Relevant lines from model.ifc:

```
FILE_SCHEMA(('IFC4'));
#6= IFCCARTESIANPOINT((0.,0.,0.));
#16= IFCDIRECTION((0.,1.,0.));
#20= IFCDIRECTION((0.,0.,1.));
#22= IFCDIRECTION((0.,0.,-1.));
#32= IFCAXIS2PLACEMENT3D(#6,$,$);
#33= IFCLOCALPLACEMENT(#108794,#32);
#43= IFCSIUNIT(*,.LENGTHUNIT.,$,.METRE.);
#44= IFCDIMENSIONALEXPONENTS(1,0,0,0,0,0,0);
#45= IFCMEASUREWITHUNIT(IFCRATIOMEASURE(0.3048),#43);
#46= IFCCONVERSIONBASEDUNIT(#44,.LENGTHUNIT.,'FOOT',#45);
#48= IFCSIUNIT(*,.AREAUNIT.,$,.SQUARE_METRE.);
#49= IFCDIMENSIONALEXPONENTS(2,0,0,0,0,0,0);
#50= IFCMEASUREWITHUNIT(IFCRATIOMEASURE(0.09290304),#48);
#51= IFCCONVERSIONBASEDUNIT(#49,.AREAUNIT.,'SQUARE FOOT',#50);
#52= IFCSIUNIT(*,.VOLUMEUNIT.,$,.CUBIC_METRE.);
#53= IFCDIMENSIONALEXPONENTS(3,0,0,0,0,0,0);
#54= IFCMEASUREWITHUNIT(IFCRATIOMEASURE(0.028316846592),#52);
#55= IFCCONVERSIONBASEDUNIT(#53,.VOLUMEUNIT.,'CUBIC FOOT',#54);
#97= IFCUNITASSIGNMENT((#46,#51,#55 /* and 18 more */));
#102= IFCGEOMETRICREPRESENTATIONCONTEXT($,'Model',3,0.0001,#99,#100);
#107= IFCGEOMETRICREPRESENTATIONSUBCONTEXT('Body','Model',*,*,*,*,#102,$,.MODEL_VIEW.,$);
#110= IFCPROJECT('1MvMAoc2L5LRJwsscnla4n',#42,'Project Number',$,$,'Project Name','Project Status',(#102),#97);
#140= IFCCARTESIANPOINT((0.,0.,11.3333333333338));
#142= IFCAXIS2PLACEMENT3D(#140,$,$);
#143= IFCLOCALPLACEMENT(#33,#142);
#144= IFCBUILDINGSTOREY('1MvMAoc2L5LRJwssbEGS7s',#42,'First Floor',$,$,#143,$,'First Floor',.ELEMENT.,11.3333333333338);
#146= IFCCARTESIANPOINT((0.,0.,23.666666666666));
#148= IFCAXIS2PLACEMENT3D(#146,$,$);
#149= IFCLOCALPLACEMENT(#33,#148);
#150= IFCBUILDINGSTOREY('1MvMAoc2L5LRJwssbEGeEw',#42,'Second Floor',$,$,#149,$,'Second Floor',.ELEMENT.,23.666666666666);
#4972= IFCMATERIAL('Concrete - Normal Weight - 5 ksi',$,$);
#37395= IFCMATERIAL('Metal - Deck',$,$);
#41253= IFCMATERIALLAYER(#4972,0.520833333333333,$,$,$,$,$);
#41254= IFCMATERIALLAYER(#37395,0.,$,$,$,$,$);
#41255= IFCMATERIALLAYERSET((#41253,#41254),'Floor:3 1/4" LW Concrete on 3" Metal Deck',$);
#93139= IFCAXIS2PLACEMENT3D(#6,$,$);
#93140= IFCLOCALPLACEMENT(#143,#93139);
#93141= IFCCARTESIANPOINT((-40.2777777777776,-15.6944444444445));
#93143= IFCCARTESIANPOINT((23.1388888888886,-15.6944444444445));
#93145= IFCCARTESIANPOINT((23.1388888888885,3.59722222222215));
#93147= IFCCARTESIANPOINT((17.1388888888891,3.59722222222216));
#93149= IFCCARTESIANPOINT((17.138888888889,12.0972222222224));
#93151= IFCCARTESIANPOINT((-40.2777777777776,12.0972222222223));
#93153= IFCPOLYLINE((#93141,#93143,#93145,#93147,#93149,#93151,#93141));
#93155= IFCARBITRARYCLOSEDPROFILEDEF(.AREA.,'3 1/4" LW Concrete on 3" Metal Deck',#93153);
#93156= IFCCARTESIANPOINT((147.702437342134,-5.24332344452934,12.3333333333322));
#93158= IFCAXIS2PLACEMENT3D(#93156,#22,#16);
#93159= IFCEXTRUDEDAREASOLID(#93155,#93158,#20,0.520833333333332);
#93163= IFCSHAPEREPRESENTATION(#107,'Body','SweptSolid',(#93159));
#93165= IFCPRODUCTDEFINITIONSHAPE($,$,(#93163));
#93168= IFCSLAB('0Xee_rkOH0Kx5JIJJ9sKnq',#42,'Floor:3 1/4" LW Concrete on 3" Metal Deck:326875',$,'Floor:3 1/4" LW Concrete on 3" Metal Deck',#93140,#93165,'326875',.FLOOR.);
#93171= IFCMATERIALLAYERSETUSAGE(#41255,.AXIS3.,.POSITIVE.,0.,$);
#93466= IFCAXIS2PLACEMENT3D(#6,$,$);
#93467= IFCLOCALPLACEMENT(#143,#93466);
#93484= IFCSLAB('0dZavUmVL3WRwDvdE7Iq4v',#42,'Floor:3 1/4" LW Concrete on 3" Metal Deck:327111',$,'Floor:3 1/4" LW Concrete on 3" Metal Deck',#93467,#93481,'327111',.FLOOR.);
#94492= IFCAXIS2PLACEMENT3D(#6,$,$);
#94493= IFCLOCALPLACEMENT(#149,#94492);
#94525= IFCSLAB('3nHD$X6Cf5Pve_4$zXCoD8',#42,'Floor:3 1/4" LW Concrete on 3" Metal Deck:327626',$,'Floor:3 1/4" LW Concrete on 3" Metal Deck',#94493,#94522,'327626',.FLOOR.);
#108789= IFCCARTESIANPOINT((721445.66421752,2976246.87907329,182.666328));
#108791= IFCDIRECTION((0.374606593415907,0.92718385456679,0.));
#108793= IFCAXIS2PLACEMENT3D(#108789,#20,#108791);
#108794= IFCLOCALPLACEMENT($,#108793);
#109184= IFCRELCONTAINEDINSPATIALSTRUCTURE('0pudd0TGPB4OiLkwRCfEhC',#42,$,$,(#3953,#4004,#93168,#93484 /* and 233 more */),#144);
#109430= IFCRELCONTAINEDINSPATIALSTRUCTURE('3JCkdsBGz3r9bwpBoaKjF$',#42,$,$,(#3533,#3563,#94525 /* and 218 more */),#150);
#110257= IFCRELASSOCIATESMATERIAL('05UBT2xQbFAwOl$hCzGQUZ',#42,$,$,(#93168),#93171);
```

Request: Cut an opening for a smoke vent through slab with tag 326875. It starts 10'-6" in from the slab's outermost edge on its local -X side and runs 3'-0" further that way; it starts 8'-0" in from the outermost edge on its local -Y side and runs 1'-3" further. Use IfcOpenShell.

```python
import numpy as np
import ifcopenshell
import ifcopenshell.api.feature
import ifcopenshell.api.geometry
import ifcopenshell.api.root
import ifcopenshell.geom
import ifcopenshell.util.placement
import ifcopenshell.util.representation
import ifcopenshell.util.shape
import ifcopenshell.util.unit

model = ifcopenshell.open("model.ifc")
unit_scale = ifcopenshell.util.unit.calculate_unit_scale(model)
settings = ifcopenshell.geom.settings()


def volume(element):
    """Net volume in cubic metres, openings subtracted."""
    shape = ifcopenshell.geom.create_shape(settings, element)
    return ifcopenshell.util.shape.get_volume(shape.geometry)


slab = model.by_id(93168)
before = volume(slab)

# Extent in the slab's own axes, in metres. The edges named are its -X and -Y sides.
slab_shape = ifcopenshell.geom.create_shape(settings, slab)
vertices = ifcopenshell.util.shape.get_vertices(slab_shape.geometry)
x_min, y_min, bottom = vertices.min(axis=0)
top = vertices[:, 2].max()

opening = ifcopenshell.api.root.create_entity(model, ifc_class="IfcOpeningElement", name="Smoke vent opening", predefined_type="OPENING")
context = ifcopenshell.util.representation.get_context(model, "Model", "Body", "MODEL_VIEW")
width, depth = 0.9144, 0.381
outline = [(0.0, 0.0), (width, 0.0), (width, depth), (0.0, depth), (0.0, 0.0)]
# Overshoot both faces by 50 mm so the cut is clean.
shape = ifcopenshell.api.geometry.add_slab_representation(
    model, context=context, depth=top - bottom + 0.1, polyline=outline
)
ifcopenshell.api.geometry.assign_representation(model, product=opening, representation=shape)

matrix = ifcopenshell.util.placement.get_local_placement(slab.ObjectPlacement)
matrix[:, 3] = matrix @ np.append(np.array([x_min + 3.2004, y_min + 2.4384, bottom - 0.05]) / unit_scale, 1.0)
ifcopenshell.api.geometry.edit_object_placement(model, product=opening, matrix=matrix, is_si=False)
ifcopenshell.api.feature.add_feature(model, feature=opening, element=slab)

after = volume(slab)

print(f"slab volume {before:.3f} -> {after:.3f} m3")

model.write("model_updated.ifc")
```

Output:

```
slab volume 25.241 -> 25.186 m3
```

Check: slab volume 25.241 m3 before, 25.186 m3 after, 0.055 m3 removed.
